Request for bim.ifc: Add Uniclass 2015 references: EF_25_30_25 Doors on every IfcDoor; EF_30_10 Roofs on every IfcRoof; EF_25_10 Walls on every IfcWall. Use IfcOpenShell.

First a look at what the model holds.

```python
import ifcopenshell

model = ifcopenshell.open("bim.ifc")
print(model.schema)
print("classifications:", [c.Name for c in model.by_type("IfcClassification")])
for ifc_class in ("IfcDoor", "IfcRoof", "IfcStair", "IfcWall", "IfcWindow"):
    print(ifc_class, len(model.by_type(ifc_class)))
```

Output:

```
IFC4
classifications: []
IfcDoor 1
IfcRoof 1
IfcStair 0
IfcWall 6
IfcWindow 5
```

```python
import ifcopenshell
import ifcopenshell.api.classification

model = ifcopenshell.open("bim.ifc")

system = ifcopenshell.api.classification.add_classification(model, classification="Uniclass 2015")

codes = {
    "IfcDoor": ("EF_25_30_25", "Doors"),
    "IfcRoof": ("EF_30_10", "Roofs"),
    "IfcWall": ("EF_25_10", "Walls"),
}
for ifc_class, (code, name) in codes.items():
    products = model.by_type(ifc_class)
    ifcopenshell.api.classification.add_reference(
        model, products=products, classification=system, identification=code, name=name
    )
    print(code, len(products))

model.write("bim_v2.ifc")
```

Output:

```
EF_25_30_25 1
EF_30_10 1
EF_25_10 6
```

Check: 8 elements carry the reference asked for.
